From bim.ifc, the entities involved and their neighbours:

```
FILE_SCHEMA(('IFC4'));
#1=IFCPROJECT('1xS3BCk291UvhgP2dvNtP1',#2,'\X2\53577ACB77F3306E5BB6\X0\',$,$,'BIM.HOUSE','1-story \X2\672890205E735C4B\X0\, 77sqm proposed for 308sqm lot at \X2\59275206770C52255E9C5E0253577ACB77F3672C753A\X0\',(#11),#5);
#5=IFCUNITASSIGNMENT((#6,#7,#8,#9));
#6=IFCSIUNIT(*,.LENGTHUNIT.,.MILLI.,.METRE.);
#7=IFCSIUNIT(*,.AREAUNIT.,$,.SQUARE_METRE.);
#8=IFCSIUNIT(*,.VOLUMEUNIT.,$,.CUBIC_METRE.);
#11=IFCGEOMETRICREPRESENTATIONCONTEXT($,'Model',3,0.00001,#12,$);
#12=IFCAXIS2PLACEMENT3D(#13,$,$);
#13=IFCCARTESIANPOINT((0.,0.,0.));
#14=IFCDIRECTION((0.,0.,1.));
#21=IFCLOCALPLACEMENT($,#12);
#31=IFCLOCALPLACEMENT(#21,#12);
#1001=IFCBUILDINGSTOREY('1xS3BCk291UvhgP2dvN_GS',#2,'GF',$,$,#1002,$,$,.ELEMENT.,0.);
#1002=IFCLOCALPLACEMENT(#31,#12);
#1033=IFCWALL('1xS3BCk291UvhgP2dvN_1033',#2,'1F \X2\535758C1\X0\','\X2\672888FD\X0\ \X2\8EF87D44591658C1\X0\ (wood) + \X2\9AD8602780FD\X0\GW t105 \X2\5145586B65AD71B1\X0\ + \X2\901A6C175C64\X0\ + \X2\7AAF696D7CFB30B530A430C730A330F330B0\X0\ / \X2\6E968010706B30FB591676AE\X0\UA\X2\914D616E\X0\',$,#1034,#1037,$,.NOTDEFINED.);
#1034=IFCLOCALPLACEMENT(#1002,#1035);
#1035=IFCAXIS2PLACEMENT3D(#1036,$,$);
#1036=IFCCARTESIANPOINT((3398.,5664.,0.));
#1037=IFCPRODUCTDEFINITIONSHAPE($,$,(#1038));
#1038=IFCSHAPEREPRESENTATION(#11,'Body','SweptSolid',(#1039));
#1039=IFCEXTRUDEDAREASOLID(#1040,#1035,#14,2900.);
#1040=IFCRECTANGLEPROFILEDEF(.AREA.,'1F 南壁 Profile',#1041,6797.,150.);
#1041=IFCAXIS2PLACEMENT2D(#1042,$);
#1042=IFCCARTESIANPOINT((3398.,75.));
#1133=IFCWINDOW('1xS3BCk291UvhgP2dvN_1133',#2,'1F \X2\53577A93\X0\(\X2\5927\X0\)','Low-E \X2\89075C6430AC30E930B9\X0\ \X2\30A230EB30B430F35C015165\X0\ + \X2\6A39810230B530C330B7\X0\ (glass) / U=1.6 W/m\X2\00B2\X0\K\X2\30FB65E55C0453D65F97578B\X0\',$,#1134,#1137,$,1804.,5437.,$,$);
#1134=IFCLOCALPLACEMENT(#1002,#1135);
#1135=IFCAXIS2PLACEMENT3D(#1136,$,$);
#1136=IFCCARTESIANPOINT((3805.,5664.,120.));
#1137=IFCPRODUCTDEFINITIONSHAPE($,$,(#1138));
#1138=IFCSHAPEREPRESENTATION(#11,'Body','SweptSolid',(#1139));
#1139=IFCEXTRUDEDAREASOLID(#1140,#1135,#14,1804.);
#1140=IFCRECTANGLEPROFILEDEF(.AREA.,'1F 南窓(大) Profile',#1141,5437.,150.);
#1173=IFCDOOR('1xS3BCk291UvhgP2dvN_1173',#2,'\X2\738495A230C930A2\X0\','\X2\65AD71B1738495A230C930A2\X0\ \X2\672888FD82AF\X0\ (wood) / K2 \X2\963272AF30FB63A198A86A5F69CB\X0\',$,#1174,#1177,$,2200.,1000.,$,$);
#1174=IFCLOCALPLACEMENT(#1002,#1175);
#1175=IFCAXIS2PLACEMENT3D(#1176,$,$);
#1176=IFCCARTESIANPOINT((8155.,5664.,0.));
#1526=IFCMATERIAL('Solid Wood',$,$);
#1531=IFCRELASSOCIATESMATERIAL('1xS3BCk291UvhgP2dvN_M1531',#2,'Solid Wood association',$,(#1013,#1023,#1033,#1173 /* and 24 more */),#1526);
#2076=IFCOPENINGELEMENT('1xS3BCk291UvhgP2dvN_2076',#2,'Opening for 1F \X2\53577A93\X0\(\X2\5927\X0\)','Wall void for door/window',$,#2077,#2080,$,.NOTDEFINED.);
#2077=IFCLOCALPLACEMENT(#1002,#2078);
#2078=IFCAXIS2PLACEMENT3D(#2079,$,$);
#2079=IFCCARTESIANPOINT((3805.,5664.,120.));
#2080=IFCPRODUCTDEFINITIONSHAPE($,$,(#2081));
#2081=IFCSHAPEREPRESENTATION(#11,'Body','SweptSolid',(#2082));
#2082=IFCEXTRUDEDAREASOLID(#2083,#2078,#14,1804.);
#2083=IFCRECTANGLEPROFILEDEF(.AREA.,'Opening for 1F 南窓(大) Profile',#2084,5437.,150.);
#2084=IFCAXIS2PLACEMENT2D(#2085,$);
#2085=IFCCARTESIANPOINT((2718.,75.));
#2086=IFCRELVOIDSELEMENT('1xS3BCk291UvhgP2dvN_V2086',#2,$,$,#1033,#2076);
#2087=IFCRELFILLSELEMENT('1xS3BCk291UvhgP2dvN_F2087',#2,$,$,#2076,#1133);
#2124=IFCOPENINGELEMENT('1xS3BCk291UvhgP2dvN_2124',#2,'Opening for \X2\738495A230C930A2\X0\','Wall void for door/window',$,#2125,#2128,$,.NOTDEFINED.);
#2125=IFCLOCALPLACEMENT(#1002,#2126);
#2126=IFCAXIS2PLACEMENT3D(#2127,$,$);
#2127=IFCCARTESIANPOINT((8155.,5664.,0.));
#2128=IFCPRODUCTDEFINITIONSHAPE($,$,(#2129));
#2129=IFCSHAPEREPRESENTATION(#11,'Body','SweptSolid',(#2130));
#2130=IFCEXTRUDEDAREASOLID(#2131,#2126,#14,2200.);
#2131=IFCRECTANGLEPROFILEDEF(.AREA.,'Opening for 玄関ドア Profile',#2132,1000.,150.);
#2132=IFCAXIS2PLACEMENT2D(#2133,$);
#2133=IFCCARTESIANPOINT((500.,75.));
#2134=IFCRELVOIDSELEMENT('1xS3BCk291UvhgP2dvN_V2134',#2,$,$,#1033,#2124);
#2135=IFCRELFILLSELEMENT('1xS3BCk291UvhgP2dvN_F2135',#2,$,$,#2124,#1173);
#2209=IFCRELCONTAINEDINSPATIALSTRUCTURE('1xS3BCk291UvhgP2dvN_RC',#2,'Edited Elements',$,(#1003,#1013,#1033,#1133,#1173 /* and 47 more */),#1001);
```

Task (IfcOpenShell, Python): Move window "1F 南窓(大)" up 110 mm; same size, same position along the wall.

```python
import numpy as np
import ifcopenshell
import ifcopenshell.api.geometry
import ifcopenshell.util.placement
import ifcopenshell.util.unit

model = ifcopenshell.open("bim.ifc")
unit_scale = ifcopenshell.util.unit.calculate_unit_scale(model)

window = model.by_guid("1xS3BCk291UvhgP2dvN_1133")
opening = window.FillsVoids[0].RelatingOpeningElement
dz = 0.11 / unit_scale

shift = np.array([0.0, 0.0, dz])
# The window is not placed relative to its opening, so move both.
for product in (opening, window):
    matrix = ifcopenshell.util.placement.get_local_placement(product.ObjectPlacement)
    matrix[:3, 3] += shift
    ifcopenshell.api.geometry.edit_object_placement(model, product=product, matrix=matrix, is_si=False)

print(f"moved by {dz * unit_scale:+.3f} m")

model.write("bim_v2.ifc")
```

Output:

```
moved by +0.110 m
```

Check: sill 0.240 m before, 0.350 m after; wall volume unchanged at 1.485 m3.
